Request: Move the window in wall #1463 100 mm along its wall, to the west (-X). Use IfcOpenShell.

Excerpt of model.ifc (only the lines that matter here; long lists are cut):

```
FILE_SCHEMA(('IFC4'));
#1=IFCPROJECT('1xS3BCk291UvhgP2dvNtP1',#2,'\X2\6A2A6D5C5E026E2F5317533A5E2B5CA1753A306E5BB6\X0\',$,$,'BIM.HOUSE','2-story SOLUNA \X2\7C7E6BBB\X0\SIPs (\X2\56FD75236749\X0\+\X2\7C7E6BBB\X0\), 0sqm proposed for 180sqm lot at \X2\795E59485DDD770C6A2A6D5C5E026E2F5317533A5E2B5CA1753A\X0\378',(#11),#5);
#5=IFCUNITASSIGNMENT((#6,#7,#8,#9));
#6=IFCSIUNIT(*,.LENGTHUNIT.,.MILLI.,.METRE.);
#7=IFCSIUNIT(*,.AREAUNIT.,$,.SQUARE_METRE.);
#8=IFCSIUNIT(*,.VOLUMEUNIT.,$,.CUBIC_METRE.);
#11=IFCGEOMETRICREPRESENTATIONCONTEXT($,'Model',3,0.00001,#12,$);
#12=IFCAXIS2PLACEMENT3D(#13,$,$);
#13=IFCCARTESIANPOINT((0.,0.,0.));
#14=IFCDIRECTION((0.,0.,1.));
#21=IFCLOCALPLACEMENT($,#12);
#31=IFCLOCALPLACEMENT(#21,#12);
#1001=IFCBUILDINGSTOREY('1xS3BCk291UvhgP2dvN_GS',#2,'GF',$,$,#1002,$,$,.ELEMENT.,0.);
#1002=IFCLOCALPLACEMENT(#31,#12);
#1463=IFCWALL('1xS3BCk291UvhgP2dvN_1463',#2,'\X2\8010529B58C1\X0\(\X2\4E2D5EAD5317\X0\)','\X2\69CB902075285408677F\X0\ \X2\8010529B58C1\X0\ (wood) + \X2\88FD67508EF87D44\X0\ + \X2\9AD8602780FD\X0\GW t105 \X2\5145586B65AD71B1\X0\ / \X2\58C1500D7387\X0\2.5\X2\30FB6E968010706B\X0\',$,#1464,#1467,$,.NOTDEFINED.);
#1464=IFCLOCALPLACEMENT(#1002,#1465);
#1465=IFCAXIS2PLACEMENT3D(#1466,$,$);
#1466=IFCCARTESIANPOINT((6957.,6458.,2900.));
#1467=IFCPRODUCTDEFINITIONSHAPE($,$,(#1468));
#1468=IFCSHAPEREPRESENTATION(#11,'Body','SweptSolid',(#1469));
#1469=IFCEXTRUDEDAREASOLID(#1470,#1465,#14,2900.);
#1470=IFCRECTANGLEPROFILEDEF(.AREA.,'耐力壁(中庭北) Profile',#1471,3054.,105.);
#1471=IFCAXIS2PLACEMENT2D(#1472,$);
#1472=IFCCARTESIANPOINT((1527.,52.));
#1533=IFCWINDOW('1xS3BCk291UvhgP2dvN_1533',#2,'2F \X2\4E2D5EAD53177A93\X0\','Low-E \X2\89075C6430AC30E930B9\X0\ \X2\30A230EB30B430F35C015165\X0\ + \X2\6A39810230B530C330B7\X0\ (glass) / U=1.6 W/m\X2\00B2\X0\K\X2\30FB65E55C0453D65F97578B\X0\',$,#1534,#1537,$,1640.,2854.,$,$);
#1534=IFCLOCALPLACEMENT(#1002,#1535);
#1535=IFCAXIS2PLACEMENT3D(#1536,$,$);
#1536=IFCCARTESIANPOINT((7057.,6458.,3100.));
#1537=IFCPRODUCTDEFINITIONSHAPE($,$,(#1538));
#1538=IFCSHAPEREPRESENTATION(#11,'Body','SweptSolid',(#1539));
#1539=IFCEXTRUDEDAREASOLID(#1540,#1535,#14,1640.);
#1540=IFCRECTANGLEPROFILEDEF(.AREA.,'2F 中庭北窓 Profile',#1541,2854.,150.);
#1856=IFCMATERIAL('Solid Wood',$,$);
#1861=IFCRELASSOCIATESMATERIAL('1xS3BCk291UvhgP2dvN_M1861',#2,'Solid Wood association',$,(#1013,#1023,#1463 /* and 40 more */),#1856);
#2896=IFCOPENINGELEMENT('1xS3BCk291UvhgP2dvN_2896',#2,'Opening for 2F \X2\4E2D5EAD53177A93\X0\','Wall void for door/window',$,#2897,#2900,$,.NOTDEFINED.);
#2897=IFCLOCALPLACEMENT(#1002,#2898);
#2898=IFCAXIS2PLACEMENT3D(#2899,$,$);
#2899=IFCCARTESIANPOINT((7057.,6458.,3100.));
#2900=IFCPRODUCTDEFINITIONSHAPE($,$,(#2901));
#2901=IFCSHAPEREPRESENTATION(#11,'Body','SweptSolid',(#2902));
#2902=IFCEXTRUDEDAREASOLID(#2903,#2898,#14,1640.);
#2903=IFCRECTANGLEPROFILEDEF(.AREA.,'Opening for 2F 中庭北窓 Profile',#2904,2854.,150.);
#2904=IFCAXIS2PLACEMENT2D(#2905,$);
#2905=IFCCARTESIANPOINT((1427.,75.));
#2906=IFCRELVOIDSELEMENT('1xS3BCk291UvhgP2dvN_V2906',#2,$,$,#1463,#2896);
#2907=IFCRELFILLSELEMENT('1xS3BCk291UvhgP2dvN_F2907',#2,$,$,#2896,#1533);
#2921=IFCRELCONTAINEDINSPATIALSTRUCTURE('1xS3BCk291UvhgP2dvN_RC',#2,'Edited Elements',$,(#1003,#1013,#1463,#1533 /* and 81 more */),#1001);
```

```python
import ifcopenshell
import ifcopenshell.api.geometry
import ifcopenshell.util.placement

model = ifcopenshell.open("model.ifc")

window = model.by_guid("1xS3BCk291UvhgP2dvN_1533")
opening = window.FillsVoids[0].RelatingOpeningElement
wall = opening.VoidsElements[0].RelatingBuildingElement

wall_matrix = ifcopenshell.util.placement.get_local_placement(wall.ObjectPlacement)
shift = wall_matrix[:3, 0] * -100.0
before = ifcopenshell.util.placement.get_local_placement(window.ObjectPlacement)[:3, 3].copy()

# The window is not placed relative to its opening, so move both.
for product in (opening, window):
    matrix = ifcopenshell.util.placement.get_local_placement(product.ObjectPlacement)
    matrix[:3, 3] += shift
    ifcopenshell.api.geometry.edit_object_placement(model, product=product, matrix=matrix, is_si=False)

after = ifcopenshell.util.placement.get_local_placement(window.ObjectPlacement)[:3, 3]
print("window moved by", (after - before).round(3) + 0.0)

model.write("model-out.ifc")
```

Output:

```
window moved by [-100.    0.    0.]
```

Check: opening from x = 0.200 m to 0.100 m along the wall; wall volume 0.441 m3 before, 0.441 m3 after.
